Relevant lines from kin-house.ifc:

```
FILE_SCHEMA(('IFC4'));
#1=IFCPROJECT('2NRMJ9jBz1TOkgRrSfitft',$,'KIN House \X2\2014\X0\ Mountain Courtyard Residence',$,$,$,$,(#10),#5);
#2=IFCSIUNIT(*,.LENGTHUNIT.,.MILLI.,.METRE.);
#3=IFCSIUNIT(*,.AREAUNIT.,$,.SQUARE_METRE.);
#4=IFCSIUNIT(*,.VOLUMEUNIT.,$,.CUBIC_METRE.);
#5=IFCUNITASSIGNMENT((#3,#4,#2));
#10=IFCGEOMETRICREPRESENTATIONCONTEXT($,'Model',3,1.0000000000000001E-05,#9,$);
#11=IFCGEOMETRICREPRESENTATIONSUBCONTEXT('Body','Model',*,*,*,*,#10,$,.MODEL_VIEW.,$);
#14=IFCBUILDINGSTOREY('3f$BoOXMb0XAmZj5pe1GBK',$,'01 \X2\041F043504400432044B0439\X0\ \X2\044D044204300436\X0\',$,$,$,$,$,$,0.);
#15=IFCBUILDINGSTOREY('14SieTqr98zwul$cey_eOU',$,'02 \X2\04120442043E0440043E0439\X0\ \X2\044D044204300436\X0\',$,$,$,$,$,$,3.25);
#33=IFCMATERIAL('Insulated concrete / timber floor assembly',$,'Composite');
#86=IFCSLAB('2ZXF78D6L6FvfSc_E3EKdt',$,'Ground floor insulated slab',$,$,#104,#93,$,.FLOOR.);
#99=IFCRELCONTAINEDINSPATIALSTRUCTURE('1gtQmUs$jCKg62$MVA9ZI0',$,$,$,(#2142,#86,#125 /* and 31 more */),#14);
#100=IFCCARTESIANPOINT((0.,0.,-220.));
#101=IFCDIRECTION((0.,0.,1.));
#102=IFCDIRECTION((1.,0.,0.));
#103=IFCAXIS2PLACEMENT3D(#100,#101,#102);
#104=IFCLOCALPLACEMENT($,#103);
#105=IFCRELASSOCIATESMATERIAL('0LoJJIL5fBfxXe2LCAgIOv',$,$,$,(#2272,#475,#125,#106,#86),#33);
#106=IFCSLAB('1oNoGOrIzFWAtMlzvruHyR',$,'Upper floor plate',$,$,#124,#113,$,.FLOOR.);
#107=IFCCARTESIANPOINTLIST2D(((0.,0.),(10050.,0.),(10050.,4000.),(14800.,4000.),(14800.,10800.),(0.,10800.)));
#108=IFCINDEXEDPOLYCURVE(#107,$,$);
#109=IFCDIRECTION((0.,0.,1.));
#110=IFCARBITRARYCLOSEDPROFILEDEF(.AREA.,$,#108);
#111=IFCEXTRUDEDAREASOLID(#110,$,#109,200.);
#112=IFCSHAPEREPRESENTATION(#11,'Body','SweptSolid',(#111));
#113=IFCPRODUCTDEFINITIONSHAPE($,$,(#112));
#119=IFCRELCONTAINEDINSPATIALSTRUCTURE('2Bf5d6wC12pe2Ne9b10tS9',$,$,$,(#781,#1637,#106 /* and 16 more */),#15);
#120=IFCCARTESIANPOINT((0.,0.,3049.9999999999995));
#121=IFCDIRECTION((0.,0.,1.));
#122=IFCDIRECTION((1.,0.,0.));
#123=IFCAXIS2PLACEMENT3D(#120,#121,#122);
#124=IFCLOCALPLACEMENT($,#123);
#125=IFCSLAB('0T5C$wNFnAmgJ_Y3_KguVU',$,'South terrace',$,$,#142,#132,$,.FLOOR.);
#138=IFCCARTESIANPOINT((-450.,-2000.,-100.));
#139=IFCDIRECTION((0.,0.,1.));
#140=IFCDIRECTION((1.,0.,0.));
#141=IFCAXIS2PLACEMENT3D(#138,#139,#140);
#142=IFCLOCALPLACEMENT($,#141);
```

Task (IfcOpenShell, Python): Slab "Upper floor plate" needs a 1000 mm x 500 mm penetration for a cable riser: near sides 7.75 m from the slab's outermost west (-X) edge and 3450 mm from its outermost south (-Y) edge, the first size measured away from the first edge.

```python
import numpy as np
import ifcopenshell
import ifcopenshell.api.feature
import ifcopenshell.api.geometry
import ifcopenshell.api.root
import ifcopenshell.geom
import ifcopenshell.util.placement
import ifcopenshell.util.representation
import ifcopenshell.util.shape
import ifcopenshell.util.unit

model = ifcopenshell.open("kin-house.ifc")
unit_scale = ifcopenshell.util.unit.calculate_unit_scale(model)
settings = ifcopenshell.geom.settings()


def volume(element):
    """Net volume in cubic metres, openings subtracted."""
    shape = ifcopenshell.geom.create_shape(settings, element)
    return ifcopenshell.util.shape.get_volume(shape.geometry)


slab = model.by_guid("1oNoGOrIzFWAtMlzvruHyR")
before = volume(slab)

# Extent in the slab's own axes, in metres. The edges named are its -X and -Y sides.
slab_shape = ifcopenshell.geom.create_shape(settings, slab)
vertices = ifcopenshell.util.shape.get_vertices(slab_shape.geometry)
x_min, y_min, bottom = vertices.min(axis=0)
top = vertices[:, 2].max()

opening = ifcopenshell.api.root.create_entity(model, ifc_class="IfcOpeningElement", name="Cable riser opening", predefined_type="OPENING")
context = ifcopenshell.util.representation.get_context(model, "Model", "Body", "MODEL_VIEW")
width, depth = 1, 0.5
outline = [(0.0, 0.0), (width, 0.0), (width, depth), (0.0, depth), (0.0, 0.0)]
# Overshoot both faces by 50 mm so the cut is clean.
shape = ifcopenshell.api.geometry.add_slab_representation(
    model, context=context, depth=top - bottom + 0.1, polyline=outline
)
ifcopenshell.api.geometry.assign_representation(model, product=opening, representation=shape)

matrix = ifcopenshell.util.placement.get_local_placement(slab.ObjectPlacement)
matrix[:, 3] = matrix @ np.append(np.array([x_min + 7.75, y_min + 3.45, bottom - 0.05]) / unit_scale, 1.0)
ifcopenshell.api.geometry.edit_object_placement(model, product=opening, matrix=matrix, is_si=False)
ifcopenshell.api.feature.add_feature(model, feature=opening, element=slab)

after = volume(slab)

print(f"slab volume {before:.3f} -> {after:.3f} m3")

model.write("kin-house_rev.ifc")
```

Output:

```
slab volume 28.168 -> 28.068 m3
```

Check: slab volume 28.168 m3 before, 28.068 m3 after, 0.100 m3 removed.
